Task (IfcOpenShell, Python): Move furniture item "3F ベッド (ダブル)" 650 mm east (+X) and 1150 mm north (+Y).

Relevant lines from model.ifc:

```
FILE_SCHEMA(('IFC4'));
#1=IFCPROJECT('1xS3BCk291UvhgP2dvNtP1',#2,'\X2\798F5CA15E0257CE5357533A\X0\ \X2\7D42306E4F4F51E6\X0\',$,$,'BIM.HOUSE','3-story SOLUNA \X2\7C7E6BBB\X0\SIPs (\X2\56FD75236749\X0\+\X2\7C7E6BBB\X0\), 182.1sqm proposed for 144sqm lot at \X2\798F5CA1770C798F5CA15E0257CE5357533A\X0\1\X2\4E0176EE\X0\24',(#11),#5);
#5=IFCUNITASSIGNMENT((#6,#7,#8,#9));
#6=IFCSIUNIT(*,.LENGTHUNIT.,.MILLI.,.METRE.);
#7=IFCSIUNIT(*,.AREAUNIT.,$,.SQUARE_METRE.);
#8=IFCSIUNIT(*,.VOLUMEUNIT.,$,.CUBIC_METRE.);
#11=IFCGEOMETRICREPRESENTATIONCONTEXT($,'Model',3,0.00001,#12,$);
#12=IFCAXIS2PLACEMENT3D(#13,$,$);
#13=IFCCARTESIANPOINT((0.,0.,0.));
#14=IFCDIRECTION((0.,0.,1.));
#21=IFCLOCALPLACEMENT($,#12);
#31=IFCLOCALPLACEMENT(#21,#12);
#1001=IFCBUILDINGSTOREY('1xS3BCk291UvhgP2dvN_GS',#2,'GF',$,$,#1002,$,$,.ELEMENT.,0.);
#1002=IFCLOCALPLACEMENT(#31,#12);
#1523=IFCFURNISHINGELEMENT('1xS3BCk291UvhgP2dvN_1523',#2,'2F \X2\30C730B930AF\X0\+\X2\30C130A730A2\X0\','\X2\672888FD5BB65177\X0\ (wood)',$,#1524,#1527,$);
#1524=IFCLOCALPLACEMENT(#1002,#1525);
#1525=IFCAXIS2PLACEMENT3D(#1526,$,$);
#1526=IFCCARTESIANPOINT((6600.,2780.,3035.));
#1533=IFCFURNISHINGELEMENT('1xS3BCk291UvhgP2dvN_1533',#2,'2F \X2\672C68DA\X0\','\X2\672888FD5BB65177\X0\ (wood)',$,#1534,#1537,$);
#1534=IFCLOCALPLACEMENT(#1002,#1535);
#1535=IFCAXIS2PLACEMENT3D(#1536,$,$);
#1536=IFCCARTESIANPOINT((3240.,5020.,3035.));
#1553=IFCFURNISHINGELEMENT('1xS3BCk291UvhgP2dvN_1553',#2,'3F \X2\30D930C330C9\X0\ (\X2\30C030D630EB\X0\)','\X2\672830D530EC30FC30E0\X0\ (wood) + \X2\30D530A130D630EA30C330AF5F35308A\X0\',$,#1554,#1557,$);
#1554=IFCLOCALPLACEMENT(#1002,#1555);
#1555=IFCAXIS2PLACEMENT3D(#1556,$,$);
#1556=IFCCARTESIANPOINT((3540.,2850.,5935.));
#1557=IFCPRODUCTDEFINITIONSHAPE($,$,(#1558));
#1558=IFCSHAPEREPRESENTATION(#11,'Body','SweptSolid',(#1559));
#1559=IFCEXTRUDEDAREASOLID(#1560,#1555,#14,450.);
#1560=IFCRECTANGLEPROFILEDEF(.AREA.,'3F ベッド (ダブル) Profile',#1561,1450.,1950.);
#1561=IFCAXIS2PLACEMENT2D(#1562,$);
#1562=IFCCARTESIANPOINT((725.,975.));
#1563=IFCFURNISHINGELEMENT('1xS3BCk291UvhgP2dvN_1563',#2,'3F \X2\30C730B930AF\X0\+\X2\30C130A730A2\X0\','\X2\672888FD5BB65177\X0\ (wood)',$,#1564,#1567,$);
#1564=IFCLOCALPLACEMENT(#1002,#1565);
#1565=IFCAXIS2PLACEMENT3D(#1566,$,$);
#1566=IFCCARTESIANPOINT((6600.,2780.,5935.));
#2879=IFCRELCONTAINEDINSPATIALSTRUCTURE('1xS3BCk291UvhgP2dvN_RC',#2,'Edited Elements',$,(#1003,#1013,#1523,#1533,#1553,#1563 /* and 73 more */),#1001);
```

```python
import ifcopenshell
import ifcopenshell.api.geometry
import ifcopenshell.util.placement
import ifcopenshell.util.unit

model = ifcopenshell.open("model.ifc")
unit_scale = ifcopenshell.util.unit.calculate_unit_scale(model)

item = model.by_id(1553)
matrix = ifcopenshell.util.placement.get_local_placement(item.ObjectPlacement)
matrix[0, 3] += 0.65 / unit_scale
matrix[1, 3] += 1.15 / unit_scale
ifcopenshell.api.geometry.edit_object_placement(model, product=item, matrix=matrix, is_si=False)

print(ifcopenshell.util.placement.get_local_placement(item.ObjectPlacement).round(3) + 0.0)

model.write("model_rev.ifc")
```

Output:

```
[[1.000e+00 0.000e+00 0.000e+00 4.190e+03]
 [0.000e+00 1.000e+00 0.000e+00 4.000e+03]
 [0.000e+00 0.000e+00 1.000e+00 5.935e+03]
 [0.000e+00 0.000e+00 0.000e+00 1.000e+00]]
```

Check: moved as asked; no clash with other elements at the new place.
